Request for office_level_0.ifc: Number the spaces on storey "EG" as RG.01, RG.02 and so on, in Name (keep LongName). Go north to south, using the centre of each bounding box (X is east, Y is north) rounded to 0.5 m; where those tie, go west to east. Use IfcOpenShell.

First a look at what the model holds.

```python
import ifcopenshell
import ifcopenshell.util.element
import ifcopenshell.util.placement

model = ifcopenshell.open("office_level_0.ifc")
print(model.schema)
storey = next(s for s in model.by_type("IfcBuildingStorey") if s.Name == "EG")
spaces = [e for e in ifcopenshell.util.element.get_decomposition(storey) if e.is_a("IfcSpace")]
for e in sorted(spaces, key=lambda e: e.id()):
    origin = ifcopenshell.util.placement.get_local_placement(e.ObjectPlacement)[:3, 3]
    print(e.id(), e.Name, e.LongName, origin.round(2) + 0.0, sep=" | ")
```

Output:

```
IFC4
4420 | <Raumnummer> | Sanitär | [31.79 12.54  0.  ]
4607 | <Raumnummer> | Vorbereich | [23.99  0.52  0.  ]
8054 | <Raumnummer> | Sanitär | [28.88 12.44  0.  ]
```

```python
import ifcopenshell
import ifcopenshell.geom
import ifcopenshell.util.element
import ifcopenshell.util.shape

model = ifcopenshell.open("office_level_0.ifc")
settings = ifcopenshell.geom.settings()
settings.set("use-world-coords", True)


def centre(element):
    shape = ifcopenshell.geom.create_shape(settings, element)
    return ifcopenshell.util.shape.get_bbox_centroid(shape.geometry)


storey = next(s for s in model.by_type("IfcBuildingStorey") if s.Name == "EG")
spaces = [e for e in ifcopenshell.util.element.get_decomposition(storey) if e.is_a("IfcSpace")]

# Insertion points can sit at a corner or the storey origin, so sort by the geometry (in metres).
centres = {e: centre(e) for e in spaces}
spaces.sort(key=lambda e: (-round(centres[e][1] / 0.5), centres[e][0]))

for i, e in enumerate(spaces, start=1):
    number = f"RG.{i:02d}"
    e.Name = number
    print(e.id(), number)

model.write("office_level_0-out.ifc")
```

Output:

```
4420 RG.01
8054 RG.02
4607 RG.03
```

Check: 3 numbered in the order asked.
